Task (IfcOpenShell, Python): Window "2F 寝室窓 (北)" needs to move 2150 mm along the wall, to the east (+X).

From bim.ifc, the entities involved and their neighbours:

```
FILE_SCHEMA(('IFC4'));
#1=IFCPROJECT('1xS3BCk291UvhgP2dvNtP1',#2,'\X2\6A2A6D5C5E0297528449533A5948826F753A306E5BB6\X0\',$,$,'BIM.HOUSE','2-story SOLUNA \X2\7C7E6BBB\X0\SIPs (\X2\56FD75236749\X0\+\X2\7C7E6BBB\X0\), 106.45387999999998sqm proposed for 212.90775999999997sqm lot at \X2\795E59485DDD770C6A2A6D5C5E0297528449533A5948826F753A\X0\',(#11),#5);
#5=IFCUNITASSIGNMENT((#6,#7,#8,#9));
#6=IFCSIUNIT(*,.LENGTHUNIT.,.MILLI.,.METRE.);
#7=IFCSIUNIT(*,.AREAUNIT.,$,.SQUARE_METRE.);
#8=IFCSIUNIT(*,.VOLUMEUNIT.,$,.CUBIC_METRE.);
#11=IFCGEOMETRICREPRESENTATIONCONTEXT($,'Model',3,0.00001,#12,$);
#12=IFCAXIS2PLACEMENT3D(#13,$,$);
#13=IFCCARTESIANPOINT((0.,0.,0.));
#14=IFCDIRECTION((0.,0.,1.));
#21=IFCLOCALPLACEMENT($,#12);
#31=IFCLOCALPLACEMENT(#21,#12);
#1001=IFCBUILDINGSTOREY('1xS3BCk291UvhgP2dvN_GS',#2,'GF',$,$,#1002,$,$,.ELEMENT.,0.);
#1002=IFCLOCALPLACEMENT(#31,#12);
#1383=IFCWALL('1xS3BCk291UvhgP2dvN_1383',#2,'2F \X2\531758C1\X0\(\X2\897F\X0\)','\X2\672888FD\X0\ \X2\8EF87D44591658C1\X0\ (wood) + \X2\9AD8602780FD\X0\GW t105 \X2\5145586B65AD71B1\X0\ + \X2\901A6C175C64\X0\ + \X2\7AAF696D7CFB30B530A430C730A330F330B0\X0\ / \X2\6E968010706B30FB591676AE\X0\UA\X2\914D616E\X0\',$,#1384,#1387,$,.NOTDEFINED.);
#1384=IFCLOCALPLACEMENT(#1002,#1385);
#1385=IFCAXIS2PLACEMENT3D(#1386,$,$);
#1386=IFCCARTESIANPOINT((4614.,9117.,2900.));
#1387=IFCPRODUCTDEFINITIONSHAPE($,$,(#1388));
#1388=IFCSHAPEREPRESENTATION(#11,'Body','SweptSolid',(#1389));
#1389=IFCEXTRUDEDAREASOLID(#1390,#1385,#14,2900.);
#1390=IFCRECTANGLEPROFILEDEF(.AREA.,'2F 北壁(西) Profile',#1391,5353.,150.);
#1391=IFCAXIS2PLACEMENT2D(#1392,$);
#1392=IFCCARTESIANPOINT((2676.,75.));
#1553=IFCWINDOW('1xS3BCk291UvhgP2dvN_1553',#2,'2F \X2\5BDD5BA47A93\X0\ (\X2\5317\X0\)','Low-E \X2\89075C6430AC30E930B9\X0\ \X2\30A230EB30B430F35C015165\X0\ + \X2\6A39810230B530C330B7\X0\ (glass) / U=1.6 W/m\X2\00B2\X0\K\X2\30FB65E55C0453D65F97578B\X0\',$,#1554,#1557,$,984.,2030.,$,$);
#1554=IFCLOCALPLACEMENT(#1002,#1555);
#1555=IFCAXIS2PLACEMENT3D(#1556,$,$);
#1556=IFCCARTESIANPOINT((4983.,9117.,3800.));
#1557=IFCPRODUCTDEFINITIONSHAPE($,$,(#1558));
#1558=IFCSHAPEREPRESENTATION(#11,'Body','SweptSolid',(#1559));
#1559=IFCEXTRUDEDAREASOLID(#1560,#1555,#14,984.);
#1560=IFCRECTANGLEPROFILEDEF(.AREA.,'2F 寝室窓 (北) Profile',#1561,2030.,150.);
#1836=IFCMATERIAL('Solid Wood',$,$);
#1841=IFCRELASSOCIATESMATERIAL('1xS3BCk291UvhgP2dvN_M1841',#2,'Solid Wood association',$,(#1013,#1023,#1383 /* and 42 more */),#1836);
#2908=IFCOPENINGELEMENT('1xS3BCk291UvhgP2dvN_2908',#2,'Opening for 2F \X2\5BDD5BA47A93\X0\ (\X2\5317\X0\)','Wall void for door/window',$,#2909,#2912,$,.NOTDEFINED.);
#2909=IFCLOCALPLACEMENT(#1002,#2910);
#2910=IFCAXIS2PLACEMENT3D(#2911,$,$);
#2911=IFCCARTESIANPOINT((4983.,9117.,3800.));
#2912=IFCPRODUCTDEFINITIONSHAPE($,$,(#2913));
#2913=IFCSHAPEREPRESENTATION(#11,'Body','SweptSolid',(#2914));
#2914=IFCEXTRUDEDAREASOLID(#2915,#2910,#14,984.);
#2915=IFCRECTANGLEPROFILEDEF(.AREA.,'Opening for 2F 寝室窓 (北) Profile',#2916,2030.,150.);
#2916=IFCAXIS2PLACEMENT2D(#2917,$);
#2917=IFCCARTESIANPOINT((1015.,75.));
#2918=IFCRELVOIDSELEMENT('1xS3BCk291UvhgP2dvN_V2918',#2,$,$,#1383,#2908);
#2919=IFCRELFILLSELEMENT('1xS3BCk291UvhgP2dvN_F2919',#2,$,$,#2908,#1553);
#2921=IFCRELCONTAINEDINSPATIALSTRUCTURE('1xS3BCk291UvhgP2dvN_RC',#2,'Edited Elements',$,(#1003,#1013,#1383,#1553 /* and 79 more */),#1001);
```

```python
import ifcopenshell
import ifcopenshell.api.geometry
import ifcopenshell.util.placement

model = ifcopenshell.open("bim.ifc")

window = model.by_guid("1xS3BCk291UvhgP2dvN_1553")
opening = window.FillsVoids[0].RelatingOpeningElement
wall = opening.VoidsElements[0].RelatingBuildingElement

wall_matrix = ifcopenshell.util.placement.get_local_placement(wall.ObjectPlacement)
shift = wall_matrix[:3, 0] * 2150.0
before = ifcopenshell.util.placement.get_local_placement(window.ObjectPlacement)[:3, 3].copy()

# The window is not placed relative to its opening, so move both.
for product in (opening, window):
    matrix = ifcopenshell.util.placement.get_local_placement(product.ObjectPlacement)
    matrix[:3, 3] += shift
    ifcopenshell.api.geometry.edit_object_placement(model, product=product, matrix=matrix, is_si=False)

after = ifcopenshell.util.placement.get_local_placement(window.ObjectPlacement)[:3, 3]
print("window moved by", (after - before).round(3) + 0.0)

model.write("bim_updated.ifc")
```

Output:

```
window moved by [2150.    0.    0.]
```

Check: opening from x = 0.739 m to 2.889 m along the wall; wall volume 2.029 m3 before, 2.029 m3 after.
